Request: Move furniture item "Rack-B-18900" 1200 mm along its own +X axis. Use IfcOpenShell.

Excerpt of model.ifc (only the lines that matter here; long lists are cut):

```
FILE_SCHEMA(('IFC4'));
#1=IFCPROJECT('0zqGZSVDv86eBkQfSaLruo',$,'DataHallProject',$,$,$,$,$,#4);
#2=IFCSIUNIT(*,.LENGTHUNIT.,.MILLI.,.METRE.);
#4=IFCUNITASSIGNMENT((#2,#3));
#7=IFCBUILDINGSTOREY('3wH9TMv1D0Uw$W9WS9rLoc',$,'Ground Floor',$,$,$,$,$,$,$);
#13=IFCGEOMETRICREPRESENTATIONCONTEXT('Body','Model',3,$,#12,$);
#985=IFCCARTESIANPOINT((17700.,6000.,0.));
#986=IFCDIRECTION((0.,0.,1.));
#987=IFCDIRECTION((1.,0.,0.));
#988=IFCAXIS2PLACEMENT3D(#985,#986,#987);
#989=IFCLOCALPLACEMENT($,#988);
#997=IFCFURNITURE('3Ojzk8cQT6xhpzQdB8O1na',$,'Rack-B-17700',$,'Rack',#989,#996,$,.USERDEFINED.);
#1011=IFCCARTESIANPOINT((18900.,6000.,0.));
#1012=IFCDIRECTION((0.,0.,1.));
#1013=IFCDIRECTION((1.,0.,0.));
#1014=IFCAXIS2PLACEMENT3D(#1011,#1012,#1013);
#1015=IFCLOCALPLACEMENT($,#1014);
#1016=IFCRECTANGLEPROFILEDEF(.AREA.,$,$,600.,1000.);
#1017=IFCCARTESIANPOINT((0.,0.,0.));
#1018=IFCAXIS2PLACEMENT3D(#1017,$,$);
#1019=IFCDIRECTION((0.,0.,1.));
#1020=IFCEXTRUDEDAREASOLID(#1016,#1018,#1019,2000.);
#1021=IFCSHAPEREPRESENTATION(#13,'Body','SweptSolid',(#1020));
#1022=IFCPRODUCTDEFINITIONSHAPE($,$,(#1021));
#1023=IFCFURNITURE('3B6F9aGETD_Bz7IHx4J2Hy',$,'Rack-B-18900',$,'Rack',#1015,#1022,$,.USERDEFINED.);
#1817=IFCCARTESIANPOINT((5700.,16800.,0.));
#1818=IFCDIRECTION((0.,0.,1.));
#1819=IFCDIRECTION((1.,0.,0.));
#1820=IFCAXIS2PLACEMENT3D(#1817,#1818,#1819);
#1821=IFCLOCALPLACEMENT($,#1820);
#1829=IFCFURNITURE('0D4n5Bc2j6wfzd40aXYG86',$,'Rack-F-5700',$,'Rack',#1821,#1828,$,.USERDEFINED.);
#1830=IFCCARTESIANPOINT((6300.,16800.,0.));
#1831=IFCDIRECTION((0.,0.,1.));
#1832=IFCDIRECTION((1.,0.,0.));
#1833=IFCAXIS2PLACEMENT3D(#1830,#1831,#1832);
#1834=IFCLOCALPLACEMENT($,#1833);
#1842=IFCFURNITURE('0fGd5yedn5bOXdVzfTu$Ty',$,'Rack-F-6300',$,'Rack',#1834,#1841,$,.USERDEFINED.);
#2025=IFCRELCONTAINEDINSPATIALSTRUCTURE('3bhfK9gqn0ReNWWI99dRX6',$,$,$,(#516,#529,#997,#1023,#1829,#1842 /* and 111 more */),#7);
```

```python
import ifcopenshell
import ifcopenshell.api.geometry
import ifcopenshell.util.placement
import ifcopenshell.util.unit

model = ifcopenshell.open("model.ifc")
unit_scale = ifcopenshell.util.unit.calculate_unit_scale(model)

item = model.by_guid("3B6F9aGETD_Bz7IHx4J2Hy")
matrix = ifcopenshell.util.placement.get_local_placement(item.ObjectPlacement)
matrix[:3, 3] += matrix[:3, 0] * 1.2 / unit_scale
ifcopenshell.api.geometry.edit_object_placement(model, product=item, matrix=matrix, is_si=False)

print(ifcopenshell.util.placement.get_local_placement(item.ObjectPlacement).round(3) + 0.0)

model.write("model_v2.ifc")
```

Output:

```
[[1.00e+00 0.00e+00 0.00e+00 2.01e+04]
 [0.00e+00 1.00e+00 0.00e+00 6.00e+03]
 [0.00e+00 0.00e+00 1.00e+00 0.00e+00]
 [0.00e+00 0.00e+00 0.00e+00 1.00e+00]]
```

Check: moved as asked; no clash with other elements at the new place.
